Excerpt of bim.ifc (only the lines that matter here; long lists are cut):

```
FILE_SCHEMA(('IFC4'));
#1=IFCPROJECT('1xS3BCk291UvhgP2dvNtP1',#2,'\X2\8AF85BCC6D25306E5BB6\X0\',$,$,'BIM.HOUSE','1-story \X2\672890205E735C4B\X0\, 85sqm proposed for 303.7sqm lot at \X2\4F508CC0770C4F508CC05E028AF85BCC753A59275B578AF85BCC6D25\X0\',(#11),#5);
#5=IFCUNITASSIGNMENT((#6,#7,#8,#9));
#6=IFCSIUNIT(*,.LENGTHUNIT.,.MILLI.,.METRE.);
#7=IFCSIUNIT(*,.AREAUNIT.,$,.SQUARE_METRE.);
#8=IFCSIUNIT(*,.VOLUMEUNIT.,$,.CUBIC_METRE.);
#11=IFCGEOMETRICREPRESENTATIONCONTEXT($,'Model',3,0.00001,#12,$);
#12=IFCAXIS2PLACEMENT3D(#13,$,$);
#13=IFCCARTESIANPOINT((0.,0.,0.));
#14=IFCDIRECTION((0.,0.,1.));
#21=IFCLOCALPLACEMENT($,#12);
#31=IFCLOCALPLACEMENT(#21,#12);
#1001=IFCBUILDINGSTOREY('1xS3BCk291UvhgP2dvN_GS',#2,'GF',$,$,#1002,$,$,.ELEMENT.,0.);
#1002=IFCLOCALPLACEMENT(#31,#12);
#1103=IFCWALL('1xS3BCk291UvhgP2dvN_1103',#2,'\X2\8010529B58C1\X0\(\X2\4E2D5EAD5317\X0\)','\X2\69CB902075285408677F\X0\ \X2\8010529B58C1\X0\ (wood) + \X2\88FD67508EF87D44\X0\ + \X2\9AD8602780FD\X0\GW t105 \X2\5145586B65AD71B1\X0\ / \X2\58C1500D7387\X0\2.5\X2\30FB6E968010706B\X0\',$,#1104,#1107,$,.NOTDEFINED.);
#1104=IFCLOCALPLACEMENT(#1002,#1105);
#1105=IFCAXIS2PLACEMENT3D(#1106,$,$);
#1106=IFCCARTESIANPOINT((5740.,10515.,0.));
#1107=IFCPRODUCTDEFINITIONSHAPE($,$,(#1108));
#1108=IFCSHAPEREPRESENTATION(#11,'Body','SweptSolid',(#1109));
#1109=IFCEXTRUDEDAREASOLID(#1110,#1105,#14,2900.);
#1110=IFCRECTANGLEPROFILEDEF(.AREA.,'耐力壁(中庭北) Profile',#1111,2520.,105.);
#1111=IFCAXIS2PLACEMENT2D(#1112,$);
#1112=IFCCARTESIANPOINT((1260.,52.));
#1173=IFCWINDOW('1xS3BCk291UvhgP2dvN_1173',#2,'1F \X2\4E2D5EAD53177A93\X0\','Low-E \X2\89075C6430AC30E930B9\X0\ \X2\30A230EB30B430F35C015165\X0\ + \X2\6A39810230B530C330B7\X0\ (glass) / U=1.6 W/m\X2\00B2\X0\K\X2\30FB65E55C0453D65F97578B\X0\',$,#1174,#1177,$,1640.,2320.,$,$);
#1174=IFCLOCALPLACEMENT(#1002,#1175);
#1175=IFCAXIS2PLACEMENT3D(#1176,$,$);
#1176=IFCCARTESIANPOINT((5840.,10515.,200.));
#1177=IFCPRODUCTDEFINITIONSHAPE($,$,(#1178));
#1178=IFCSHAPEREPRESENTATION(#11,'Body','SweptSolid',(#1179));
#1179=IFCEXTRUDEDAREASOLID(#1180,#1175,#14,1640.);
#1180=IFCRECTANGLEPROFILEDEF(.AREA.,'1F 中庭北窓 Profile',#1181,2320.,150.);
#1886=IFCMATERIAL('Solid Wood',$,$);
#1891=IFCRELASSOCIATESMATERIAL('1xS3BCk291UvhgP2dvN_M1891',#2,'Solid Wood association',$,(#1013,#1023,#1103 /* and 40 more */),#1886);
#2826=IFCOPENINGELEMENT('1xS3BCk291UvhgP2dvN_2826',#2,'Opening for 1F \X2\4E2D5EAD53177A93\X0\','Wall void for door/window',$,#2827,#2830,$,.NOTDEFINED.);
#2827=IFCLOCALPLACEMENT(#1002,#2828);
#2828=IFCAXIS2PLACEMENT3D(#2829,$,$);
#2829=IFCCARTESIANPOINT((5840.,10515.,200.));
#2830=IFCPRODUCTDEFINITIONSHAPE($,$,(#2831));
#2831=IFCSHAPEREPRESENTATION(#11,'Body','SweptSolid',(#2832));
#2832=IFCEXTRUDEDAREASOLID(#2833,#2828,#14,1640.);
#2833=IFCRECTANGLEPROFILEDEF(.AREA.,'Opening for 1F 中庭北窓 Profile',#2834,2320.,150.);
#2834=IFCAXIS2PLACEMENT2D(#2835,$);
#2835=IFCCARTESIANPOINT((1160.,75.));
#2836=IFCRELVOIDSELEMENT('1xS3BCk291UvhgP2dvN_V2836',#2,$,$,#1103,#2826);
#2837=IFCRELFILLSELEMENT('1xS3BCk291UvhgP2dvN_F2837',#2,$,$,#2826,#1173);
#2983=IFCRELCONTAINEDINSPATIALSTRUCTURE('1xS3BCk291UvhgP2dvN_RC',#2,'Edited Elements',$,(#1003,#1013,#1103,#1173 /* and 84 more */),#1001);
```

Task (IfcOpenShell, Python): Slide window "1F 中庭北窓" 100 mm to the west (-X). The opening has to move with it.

```python
import ifcopenshell
import ifcopenshell.api.geometry
import ifcopenshell.util.placement

model = ifcopenshell.open("bim.ifc")

window = model.by_guid("1xS3BCk291UvhgP2dvN_1173")
opening = window.FillsVoids[0].RelatingOpeningElement
wall = opening.VoidsElements[0].RelatingBuildingElement

wall_matrix = ifcopenshell.util.placement.get_local_placement(wall.ObjectPlacement)
shift = wall_matrix[:3, 0] * -100.0
before = ifcopenshell.util.placement.get_local_placement(window.ObjectPlacement)[:3, 3].copy()

# The window is not placed relative to its opening, so move both.
for product in (opening, window):
    matrix = ifcopenshell.util.placement.get_local_placement(product.ObjectPlacement)
    matrix[:3, 3] += shift
    ifcopenshell.api.geometry.edit_object_placement(model, product=product, matrix=matrix, is_si=False)

after = ifcopenshell.util.placement.get_local_placement(window.ObjectPlacement)[:3, 3]
print("window moved by", (after - before).round(3) + 0.0)

model.write("bim-out.ifc")
```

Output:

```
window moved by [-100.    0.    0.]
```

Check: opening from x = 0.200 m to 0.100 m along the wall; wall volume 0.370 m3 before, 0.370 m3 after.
